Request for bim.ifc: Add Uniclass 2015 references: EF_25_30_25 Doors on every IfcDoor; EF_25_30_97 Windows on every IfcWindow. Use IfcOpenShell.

First a look at what the model holds.

```python
import ifcopenshell

model = ifcopenshell.open("bim.ifc")
print(model.schema)
print("classifications:", [c.Name for c in model.by_type("IfcClassification")])
for ifc_class in ("IfcDoor", "IfcRoof", "IfcStair", "IfcWall", "IfcWindow"):
    print(ifc_class, len(model.by_type(ifc_class)))
```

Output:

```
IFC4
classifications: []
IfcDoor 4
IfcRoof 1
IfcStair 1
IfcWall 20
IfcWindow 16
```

```python
import ifcopenshell
import ifcopenshell.api.classification

model = ifcopenshell.open("bim.ifc")

system = ifcopenshell.api.classification.add_classification(model, classification="Uniclass 2015")

codes = {
    "IfcDoor": ("EF_25_30_25", "Doors"),
    "IfcWindow": ("EF_25_30_97", "Windows"),
}
for ifc_class, (code, name) in codes.items():
    products = model.by_type(ifc_class)
    ifcopenshell.api.classification.add_reference(
        model, products=products, classification=system, identification=code, name=name
    )
    print(code, len(products))

model.write("bim_rev.ifc")
```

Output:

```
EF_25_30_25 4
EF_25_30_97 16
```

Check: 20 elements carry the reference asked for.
